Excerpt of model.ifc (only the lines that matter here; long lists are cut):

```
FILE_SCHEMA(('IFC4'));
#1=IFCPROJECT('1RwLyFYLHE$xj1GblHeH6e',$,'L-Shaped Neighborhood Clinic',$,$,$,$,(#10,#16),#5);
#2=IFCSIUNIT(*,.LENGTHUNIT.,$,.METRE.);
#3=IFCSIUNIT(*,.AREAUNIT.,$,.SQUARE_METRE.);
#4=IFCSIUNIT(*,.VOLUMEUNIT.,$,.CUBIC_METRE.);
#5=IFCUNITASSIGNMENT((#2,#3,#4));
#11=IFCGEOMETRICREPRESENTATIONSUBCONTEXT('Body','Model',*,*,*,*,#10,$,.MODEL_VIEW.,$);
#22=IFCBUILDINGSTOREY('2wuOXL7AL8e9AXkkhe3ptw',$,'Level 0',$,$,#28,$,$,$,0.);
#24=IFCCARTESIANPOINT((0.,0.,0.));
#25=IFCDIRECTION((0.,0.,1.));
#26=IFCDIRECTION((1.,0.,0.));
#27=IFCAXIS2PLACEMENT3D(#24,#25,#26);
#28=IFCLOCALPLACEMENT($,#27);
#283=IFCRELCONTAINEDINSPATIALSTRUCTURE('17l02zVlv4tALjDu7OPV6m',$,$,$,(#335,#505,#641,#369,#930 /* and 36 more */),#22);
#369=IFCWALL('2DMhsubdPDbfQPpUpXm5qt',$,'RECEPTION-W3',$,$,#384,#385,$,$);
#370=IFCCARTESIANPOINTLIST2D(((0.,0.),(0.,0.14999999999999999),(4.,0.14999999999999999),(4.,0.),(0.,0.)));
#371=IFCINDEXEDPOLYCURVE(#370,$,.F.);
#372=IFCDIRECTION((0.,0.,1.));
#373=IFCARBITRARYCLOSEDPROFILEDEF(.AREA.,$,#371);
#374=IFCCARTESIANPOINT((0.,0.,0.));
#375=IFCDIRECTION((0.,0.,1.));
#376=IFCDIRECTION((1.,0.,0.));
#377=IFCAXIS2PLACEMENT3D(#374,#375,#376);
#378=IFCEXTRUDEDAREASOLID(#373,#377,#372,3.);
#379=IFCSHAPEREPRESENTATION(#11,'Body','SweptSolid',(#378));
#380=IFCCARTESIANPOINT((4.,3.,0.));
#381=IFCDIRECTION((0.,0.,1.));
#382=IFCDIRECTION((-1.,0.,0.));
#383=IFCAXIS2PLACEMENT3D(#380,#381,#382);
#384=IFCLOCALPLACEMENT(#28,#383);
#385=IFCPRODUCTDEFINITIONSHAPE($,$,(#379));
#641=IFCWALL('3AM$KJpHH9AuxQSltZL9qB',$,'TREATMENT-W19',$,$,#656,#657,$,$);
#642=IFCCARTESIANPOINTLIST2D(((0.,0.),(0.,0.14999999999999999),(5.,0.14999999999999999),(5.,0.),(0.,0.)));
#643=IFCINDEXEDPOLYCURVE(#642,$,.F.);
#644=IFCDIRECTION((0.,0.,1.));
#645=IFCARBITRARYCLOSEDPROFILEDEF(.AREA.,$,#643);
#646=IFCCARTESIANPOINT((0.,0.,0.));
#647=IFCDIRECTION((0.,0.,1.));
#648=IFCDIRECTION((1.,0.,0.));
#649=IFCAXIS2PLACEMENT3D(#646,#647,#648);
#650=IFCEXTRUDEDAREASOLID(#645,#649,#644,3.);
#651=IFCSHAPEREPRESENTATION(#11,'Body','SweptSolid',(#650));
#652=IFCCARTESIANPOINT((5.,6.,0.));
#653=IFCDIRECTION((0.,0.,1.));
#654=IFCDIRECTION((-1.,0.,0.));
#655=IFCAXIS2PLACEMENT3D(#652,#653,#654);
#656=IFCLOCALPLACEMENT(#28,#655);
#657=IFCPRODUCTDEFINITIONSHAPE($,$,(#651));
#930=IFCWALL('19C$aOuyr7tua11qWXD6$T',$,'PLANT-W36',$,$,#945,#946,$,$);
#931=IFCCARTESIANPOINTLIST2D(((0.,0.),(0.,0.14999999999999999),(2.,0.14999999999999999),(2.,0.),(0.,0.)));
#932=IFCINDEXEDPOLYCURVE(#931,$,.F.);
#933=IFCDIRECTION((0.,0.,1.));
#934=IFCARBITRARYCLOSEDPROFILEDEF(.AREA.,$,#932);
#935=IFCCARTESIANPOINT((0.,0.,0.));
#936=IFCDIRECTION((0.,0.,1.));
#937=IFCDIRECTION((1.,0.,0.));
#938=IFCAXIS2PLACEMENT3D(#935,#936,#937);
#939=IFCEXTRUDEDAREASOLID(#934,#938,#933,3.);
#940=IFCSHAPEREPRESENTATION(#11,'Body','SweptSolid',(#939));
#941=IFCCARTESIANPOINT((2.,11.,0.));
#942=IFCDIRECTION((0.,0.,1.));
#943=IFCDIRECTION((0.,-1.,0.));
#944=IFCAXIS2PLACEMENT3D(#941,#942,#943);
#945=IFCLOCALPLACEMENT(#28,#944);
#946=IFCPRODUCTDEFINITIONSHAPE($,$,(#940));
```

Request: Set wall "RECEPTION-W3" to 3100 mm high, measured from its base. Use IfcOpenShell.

```python
import ifcopenshell
import ifcopenshell.geom
import ifcopenshell.util.representation
import ifcopenshell.util.shape

model = ifcopenshell.open("model.ifc")
settings = ifcopenshell.geom.settings()


def volume(element):
    """Net volume in cubic metres, openings subtracted."""
    shape = ifcopenshell.geom.create_shape(settings, element)
    return ifcopenshell.util.shape.get_volume(shape.geometry)


wall = model.by_guid("2DMhsubdPDbfQPpUpXm5qt")
before = volume(wall)

body = ifcopenshell.util.representation.get_representation(wall, "Model", "Body")
solid = body.Items[0]
old_height = solid.Depth
solid.Depth = 3.1
after = volume(wall)

print(f"height {old_height:g} -> {solid.Depth:g}, volume {before:.3f} -> {after:.3f} m3")

model.write("model_updated.ifc")
```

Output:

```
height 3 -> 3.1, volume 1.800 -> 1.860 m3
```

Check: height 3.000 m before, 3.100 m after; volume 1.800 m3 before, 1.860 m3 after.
